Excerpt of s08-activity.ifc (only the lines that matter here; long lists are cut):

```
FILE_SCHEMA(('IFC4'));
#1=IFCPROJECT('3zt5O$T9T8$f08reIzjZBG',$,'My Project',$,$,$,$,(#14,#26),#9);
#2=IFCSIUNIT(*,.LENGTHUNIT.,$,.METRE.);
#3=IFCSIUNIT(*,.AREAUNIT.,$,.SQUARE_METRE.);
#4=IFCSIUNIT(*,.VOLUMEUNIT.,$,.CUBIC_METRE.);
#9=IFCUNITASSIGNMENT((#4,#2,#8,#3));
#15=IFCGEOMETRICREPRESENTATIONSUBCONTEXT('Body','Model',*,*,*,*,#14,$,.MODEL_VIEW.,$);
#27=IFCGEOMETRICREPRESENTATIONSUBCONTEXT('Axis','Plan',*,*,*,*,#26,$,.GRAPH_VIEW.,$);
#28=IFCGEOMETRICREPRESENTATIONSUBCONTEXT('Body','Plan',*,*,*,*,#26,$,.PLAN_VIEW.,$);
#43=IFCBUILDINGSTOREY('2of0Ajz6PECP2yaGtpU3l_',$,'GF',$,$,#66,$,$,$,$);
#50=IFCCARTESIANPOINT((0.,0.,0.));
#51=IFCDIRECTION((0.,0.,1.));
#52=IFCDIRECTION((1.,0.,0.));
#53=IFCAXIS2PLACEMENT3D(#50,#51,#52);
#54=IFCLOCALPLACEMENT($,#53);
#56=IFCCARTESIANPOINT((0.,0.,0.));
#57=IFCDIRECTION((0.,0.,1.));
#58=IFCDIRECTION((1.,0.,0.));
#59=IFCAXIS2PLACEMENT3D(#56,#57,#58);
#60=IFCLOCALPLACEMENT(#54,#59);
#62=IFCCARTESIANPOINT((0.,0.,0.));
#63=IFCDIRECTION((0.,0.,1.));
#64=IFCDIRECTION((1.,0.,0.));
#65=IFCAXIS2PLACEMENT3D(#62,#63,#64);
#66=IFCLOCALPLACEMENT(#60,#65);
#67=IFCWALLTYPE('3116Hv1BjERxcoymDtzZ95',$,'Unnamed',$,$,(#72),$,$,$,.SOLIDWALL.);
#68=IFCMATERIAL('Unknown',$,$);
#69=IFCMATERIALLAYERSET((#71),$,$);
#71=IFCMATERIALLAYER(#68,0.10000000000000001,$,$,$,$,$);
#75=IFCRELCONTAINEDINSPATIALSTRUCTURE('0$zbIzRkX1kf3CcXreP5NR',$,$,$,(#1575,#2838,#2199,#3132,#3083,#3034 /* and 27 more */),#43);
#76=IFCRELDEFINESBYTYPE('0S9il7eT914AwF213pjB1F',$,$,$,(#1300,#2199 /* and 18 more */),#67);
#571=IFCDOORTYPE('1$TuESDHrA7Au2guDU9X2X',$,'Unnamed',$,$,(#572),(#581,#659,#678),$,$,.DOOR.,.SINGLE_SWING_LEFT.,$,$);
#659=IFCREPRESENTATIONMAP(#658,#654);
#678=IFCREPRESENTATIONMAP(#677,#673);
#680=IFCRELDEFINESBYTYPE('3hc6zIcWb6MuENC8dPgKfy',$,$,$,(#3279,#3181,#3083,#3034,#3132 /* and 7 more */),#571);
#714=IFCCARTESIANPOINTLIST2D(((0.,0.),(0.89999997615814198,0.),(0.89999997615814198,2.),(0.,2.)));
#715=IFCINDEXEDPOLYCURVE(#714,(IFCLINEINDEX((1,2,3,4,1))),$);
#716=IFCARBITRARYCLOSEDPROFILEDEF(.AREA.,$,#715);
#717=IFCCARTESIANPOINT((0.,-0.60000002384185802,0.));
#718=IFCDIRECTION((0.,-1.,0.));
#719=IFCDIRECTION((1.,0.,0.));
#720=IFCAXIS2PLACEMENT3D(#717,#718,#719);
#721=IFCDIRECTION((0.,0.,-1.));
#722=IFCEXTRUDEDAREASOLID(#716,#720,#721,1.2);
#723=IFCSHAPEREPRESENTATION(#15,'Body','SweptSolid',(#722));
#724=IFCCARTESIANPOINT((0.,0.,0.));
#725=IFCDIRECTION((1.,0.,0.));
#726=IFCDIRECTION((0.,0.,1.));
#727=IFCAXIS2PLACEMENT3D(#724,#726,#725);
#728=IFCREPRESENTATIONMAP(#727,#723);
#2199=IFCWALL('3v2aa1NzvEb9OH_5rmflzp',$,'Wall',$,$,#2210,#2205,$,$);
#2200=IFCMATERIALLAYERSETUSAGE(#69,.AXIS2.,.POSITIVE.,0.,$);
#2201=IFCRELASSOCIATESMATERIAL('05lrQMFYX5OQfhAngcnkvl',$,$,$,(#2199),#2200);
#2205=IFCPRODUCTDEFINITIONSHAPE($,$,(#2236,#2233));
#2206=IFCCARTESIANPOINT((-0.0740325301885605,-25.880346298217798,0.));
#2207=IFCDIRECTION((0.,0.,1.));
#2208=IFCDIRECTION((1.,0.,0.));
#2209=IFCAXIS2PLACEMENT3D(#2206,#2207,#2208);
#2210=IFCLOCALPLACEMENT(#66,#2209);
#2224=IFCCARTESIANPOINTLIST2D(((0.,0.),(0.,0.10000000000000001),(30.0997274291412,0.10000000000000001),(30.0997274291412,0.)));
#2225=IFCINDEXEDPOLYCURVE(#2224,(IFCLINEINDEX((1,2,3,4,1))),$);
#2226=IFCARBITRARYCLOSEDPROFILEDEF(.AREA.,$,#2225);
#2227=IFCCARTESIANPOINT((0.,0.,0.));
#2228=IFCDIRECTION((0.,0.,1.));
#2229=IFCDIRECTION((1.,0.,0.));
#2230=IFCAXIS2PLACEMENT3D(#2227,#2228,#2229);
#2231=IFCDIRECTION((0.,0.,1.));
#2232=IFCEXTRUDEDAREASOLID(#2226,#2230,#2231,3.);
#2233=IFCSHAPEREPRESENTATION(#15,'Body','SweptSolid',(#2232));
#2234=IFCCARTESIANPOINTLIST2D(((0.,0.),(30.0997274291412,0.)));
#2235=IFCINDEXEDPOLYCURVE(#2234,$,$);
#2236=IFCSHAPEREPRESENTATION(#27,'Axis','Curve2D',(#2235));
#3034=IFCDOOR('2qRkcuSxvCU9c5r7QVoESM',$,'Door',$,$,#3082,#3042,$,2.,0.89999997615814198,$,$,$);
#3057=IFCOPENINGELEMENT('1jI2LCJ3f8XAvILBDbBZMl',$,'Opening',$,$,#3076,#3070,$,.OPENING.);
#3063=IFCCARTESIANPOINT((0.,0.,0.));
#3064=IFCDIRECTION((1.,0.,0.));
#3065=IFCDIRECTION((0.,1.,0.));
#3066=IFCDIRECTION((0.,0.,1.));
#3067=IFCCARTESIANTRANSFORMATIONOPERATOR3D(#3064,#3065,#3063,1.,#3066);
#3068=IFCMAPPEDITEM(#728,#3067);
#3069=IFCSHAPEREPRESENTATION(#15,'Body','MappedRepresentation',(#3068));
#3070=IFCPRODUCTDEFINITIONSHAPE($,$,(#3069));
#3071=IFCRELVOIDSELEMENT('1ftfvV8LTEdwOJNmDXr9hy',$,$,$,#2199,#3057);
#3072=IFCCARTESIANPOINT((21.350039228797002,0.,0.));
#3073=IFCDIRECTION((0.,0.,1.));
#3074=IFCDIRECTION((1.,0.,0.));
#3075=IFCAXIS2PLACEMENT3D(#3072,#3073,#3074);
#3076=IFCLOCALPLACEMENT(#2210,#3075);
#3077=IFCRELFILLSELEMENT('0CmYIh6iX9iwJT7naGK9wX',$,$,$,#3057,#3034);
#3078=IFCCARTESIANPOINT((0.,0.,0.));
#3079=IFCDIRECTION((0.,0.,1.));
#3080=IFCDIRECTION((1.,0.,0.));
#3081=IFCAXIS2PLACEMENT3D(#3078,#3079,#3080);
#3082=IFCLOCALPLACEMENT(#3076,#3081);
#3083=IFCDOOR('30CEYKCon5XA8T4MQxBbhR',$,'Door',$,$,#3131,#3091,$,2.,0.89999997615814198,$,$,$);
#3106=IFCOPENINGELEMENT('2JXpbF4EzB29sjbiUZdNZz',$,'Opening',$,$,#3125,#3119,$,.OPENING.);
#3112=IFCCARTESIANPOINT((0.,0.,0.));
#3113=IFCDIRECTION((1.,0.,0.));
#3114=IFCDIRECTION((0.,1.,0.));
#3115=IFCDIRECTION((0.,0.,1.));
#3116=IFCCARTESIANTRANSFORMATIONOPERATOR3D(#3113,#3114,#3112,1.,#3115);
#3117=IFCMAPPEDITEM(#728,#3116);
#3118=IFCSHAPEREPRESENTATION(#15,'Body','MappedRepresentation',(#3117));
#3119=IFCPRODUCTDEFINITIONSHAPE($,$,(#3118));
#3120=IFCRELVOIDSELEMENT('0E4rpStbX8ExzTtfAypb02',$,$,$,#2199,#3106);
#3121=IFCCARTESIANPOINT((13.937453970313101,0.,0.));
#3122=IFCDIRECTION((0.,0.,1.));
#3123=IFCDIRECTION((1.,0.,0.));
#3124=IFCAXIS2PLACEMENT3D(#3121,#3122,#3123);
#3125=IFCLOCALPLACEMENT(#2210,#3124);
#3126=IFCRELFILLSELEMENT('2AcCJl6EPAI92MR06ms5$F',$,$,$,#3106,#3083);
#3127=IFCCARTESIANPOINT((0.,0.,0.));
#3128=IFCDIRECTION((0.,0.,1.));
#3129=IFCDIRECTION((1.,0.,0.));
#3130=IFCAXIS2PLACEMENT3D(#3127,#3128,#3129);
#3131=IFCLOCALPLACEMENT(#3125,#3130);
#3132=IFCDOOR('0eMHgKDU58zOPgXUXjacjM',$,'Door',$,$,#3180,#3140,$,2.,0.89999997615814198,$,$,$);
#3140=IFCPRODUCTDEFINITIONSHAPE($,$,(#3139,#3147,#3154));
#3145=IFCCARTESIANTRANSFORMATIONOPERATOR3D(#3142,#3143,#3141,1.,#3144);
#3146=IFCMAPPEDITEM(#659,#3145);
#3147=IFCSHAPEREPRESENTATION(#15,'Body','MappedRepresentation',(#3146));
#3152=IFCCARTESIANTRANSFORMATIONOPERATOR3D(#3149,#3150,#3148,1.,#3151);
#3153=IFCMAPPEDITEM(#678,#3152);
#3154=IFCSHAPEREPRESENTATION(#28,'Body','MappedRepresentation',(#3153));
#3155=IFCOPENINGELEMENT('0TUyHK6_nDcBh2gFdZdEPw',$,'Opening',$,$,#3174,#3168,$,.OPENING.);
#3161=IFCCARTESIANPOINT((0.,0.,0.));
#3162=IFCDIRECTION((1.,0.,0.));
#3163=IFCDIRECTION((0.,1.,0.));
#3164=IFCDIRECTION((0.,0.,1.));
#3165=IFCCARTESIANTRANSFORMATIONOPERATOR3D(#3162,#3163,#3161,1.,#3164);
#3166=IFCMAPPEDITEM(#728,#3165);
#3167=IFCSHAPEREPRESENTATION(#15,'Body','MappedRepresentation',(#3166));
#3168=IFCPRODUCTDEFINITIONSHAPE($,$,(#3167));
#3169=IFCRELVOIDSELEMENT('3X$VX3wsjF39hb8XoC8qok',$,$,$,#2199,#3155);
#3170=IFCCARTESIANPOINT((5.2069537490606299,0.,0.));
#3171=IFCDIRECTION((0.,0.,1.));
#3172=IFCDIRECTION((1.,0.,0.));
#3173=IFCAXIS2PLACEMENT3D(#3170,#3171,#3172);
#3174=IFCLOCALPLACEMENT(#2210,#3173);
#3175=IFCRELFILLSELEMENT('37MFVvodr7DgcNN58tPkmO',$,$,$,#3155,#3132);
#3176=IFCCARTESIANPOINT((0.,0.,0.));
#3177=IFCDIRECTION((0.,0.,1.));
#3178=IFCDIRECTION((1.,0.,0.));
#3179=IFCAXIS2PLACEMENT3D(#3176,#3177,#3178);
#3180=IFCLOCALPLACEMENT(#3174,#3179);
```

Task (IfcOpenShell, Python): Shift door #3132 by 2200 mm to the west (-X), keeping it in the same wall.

```python
import ifcopenshell
import ifcopenshell.api.geometry
import ifcopenshell.util.placement

model = ifcopenshell.open("s08-activity.ifc")

door = model.by_guid("0eMHgKDU58zOPgXUXjacjM")
opening = door.FillsVoids[0].RelatingOpeningElement
wall = opening.VoidsElements[0].RelatingBuildingElement

wall_matrix = ifcopenshell.util.placement.get_local_placement(wall.ObjectPlacement)
shift = wall_matrix[:3, 0] * -2.2
before = ifcopenshell.util.placement.get_local_placement(door.ObjectPlacement)[:3, 3].copy()

# The door is placed relative to its opening, so it follows when the opening moves.
matrix = ifcopenshell.util.placement.get_local_placement(opening.ObjectPlacement)
matrix[:3, 3] += shift
ifcopenshell.api.geometry.edit_object_placement(
    model, product=opening, matrix=matrix, is_si=False, should_transform_children=True
)

after = ifcopenshell.util.placement.get_local_placement(door.ObjectPlacement)[:3, 3]
print("door moved by", (after - before).round(3) + 0.0)

model.write("s08-activity_rev.ifc")
```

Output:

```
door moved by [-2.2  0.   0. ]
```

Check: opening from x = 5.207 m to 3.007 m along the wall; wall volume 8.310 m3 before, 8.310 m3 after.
